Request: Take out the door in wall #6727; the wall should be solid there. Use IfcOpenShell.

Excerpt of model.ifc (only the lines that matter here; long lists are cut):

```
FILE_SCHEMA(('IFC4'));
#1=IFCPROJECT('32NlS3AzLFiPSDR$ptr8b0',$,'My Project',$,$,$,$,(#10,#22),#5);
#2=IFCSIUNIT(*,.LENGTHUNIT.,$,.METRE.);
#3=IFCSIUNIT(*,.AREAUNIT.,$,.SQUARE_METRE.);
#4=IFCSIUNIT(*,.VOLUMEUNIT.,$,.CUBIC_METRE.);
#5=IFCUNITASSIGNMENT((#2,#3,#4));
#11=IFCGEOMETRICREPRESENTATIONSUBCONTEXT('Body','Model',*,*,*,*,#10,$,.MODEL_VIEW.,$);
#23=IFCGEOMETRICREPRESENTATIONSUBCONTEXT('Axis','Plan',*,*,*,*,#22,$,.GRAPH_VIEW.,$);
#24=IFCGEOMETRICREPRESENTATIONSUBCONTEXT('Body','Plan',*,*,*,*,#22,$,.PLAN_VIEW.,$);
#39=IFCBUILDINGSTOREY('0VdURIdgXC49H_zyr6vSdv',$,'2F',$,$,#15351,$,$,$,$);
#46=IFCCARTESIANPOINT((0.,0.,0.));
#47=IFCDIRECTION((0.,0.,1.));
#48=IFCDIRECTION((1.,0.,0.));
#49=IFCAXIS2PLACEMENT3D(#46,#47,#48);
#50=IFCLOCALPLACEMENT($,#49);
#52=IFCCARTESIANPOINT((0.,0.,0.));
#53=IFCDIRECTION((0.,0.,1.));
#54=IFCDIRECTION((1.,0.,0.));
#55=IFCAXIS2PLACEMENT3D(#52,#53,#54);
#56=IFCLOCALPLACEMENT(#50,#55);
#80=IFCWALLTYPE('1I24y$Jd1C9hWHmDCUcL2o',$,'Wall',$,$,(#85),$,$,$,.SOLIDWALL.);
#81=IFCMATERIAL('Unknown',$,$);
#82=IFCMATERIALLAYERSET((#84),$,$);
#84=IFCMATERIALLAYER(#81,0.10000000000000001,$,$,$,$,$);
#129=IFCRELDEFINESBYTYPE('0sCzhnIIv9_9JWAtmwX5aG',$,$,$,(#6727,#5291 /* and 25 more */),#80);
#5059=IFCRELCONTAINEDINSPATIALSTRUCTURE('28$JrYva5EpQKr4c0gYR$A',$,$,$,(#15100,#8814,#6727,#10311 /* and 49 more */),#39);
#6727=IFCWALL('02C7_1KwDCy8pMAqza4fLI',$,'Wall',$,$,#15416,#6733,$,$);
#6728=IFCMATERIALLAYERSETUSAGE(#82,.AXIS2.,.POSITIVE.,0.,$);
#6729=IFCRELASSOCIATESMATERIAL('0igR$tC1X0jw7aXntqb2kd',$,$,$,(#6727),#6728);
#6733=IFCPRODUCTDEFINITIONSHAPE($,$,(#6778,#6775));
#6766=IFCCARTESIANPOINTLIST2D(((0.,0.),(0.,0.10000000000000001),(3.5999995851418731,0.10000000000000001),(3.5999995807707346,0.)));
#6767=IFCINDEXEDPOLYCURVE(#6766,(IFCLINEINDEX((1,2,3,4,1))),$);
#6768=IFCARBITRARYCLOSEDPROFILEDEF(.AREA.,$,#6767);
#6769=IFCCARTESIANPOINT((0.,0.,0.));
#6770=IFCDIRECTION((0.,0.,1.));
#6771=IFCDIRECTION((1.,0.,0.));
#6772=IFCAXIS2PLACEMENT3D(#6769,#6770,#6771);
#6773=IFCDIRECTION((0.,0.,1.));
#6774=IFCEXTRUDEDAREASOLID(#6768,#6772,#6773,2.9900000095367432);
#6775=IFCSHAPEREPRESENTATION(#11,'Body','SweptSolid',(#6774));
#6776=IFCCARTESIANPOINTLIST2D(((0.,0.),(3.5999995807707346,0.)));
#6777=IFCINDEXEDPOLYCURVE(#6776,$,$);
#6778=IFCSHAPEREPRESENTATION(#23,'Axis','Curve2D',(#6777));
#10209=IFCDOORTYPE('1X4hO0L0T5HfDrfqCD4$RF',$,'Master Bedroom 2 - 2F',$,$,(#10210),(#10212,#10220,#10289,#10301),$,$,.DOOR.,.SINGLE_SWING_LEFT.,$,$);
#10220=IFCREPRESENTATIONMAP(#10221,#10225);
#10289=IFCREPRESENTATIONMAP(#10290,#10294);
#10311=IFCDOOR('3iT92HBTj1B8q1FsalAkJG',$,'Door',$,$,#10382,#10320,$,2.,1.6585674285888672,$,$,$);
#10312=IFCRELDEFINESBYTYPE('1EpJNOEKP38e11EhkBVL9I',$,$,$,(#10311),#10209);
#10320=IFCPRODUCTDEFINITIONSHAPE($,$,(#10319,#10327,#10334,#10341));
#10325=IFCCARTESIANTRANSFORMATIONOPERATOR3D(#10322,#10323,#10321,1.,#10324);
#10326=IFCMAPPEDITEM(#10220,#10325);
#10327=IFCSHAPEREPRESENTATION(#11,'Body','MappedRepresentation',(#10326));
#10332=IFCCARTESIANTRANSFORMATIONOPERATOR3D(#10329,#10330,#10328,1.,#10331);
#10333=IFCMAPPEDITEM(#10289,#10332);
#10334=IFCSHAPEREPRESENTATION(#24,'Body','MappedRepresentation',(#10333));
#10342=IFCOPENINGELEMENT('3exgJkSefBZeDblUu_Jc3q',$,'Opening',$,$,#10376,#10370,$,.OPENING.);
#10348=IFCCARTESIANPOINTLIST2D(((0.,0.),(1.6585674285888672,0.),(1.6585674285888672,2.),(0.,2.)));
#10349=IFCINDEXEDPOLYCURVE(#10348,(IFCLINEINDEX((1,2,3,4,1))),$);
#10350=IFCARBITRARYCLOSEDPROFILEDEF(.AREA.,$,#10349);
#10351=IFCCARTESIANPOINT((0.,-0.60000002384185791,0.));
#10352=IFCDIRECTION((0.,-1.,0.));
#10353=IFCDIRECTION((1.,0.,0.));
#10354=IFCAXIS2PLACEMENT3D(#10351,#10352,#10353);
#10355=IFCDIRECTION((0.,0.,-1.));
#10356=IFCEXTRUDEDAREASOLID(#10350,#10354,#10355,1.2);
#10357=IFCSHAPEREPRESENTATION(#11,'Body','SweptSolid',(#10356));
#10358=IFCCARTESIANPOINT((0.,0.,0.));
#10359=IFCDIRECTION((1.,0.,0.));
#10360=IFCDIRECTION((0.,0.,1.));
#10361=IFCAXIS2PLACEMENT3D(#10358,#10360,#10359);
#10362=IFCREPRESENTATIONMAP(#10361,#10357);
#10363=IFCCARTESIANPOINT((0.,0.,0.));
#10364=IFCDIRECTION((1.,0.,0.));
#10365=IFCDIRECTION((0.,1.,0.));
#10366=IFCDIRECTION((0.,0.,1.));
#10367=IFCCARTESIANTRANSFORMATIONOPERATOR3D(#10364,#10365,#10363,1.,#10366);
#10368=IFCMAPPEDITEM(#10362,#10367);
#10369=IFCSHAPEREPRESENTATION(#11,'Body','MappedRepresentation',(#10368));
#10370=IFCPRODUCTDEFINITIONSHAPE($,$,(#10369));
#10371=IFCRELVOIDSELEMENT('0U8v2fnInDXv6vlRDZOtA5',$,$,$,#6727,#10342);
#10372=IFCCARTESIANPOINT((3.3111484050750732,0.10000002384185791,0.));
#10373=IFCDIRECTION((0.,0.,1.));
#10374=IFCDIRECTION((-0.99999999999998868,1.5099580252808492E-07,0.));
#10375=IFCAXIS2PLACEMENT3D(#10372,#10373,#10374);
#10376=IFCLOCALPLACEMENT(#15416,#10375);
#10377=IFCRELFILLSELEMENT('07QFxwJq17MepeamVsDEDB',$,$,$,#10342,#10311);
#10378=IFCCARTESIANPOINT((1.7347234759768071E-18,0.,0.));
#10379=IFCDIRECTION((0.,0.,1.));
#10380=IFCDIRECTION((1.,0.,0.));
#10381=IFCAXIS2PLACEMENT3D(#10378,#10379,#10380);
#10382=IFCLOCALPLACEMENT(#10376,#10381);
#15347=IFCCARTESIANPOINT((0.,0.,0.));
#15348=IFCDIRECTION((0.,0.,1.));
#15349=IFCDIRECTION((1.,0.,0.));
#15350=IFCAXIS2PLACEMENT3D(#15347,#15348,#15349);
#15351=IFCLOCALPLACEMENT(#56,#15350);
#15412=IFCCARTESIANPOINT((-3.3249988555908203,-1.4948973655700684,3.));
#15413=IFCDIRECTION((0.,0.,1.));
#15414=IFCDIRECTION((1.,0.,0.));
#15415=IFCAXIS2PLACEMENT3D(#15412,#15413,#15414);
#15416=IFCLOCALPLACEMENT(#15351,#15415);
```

```python
import ifcopenshell
import ifcopenshell.api.feature
import ifcopenshell.api.root
import ifcopenshell.geom
import ifcopenshell.util.shape

model = ifcopenshell.open("model.ifc")
settings = ifcopenshell.geom.settings()


def volume(element):
    """Net volume in cubic metres, openings subtracted."""
    shape = ifcopenshell.geom.create_shape(settings, element)
    return ifcopenshell.util.shape.get_volume(shape.geometry)


door = model.by_id(10311)
opening = door.FillsVoids[0].RelatingOpeningElement
wall = opening.VoidsElements[0].RelatingBuildingElement
before = volume(wall)

ifcopenshell.api.root.remove_product(model, product=door)
ifcopenshell.api.feature.remove_feature(model, feature=opening)

after = volume(wall)

print(f"wall volume {before:.3f} -> {after:.3f} m3")

model.write("model-out.ifc")
```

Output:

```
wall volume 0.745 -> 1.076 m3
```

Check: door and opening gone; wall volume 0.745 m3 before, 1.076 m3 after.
